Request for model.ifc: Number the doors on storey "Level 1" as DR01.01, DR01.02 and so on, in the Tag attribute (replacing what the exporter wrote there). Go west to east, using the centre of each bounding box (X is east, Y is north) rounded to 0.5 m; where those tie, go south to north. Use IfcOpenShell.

First a look at what the model holds.

```python
import ifcopenshell
import ifcopenshell.util.element
import ifcopenshell.util.placement

model = ifcopenshell.open("model.ifc")
print(model.schema)
storey = next(s for s in model.by_type("IfcBuildingStorey") if s.Name == "Level 1")
doors = [e for e in ifcopenshell.util.element.get_decomposition(storey) if e.is_a("IfcDoor")]
for e in sorted(doors, key=lambda e: e.id()):
    origin = ifcopenshell.util.placement.get_local_placement(e.ObjectPlacement)[:3, 3]
    print(e.id(), e.Tag, e.Name, origin.round(2) + 0.0, sep=" | ")
```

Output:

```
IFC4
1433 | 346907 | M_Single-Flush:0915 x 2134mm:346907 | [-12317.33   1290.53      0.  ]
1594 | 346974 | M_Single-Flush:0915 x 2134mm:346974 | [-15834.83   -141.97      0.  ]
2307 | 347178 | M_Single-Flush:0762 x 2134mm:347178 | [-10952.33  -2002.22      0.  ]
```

```python
import ifcopenshell
import ifcopenshell.geom
import ifcopenshell.util.element
import ifcopenshell.util.shape

model = ifcopenshell.open("model.ifc")
settings = ifcopenshell.geom.settings()
settings.set("use-world-coords", True)


def centre(element):
    shape = ifcopenshell.geom.create_shape(settings, element)
    return ifcopenshell.util.shape.get_bbox_centroid(shape.geometry)


storey = next(s for s in model.by_type("IfcBuildingStorey") if s.Name == "Level 1")
doors = [e for e in ifcopenshell.util.element.get_decomposition(storey) if e.is_a("IfcDoor")]

# Insertion points can sit at a corner or the storey origin, so sort by the geometry (in metres).
centres = {e: centre(e) for e in doors}
doors.sort(key=lambda e: (round(centres[e][0] / 0.5), centres[e][1]))

for i, e in enumerate(doors, start=1):
    number = f"DR01.{i:02d}"
    e.Tag = number
    print(e.id(), number)

model.write("model_edited.ifc")
```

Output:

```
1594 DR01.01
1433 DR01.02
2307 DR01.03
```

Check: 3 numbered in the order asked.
